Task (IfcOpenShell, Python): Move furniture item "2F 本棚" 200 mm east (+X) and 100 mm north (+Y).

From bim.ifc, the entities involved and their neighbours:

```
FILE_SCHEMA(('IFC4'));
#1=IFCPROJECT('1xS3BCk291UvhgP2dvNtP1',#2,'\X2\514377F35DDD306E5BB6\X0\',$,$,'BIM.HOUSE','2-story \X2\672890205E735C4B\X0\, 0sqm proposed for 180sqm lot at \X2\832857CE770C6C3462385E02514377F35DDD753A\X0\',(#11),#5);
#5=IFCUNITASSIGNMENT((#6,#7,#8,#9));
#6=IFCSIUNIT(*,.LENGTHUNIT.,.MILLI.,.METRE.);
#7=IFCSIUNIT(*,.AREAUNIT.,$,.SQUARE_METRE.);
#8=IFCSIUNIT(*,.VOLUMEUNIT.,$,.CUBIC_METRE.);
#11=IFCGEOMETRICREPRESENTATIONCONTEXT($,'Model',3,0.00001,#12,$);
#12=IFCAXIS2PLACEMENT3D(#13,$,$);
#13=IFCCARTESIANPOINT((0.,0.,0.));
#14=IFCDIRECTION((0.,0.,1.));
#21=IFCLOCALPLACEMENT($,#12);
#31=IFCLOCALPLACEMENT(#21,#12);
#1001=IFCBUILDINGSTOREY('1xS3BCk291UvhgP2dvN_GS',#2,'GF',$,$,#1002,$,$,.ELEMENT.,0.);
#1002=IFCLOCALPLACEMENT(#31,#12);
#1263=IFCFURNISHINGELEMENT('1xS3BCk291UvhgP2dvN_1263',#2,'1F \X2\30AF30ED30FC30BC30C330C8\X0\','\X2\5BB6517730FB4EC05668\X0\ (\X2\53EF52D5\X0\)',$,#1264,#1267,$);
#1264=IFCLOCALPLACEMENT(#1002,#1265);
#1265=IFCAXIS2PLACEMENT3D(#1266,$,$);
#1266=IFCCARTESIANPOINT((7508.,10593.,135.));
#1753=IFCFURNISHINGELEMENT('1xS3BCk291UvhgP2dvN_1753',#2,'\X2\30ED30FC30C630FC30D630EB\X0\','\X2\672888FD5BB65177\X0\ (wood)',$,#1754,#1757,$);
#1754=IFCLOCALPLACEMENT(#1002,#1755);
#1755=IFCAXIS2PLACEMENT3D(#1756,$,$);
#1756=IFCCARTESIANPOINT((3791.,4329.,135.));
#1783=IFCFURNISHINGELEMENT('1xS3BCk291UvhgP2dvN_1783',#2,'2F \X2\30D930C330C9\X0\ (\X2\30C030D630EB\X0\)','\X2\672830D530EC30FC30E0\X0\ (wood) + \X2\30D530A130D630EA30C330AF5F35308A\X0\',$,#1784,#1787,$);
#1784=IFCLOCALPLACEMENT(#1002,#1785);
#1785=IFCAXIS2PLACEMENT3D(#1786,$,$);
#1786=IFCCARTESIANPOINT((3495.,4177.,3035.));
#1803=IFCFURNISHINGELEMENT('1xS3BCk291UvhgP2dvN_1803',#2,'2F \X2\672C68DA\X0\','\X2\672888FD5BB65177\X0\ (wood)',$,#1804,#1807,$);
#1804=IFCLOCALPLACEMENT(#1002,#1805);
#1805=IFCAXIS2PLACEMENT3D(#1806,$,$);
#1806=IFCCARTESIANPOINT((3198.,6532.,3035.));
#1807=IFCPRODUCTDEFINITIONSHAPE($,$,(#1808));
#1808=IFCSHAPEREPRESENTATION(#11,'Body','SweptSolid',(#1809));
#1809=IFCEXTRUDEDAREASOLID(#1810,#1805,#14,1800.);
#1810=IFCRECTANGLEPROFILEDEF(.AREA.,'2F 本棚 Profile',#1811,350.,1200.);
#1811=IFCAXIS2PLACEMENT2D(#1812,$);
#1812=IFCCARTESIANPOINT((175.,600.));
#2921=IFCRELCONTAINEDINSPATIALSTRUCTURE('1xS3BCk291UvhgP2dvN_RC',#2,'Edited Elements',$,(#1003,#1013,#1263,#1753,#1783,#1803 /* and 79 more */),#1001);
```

```python
import ifcopenshell
import ifcopenshell.api.geometry
import ifcopenshell.util.placement
import ifcopenshell.util.unit

model = ifcopenshell.open("bim.ifc")
unit_scale = ifcopenshell.util.unit.calculate_unit_scale(model)

item = model.by_guid("1xS3BCk291UvhgP2dvN_1803")
matrix = ifcopenshell.util.placement.get_local_placement(item.ObjectPlacement)
matrix[0, 3] += 0.2 / unit_scale
matrix[1, 3] += 0.1 / unit_scale
ifcopenshell.api.geometry.edit_object_placement(model, product=item, matrix=matrix, is_si=False)

print(ifcopenshell.util.placement.get_local_placement(item.ObjectPlacement).round(3) + 0.0)

model.write("bim_edited.ifc")
```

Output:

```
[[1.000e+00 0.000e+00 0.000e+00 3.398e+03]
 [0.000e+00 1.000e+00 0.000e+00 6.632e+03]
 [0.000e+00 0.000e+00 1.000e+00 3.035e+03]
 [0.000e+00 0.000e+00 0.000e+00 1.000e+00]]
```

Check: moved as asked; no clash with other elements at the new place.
